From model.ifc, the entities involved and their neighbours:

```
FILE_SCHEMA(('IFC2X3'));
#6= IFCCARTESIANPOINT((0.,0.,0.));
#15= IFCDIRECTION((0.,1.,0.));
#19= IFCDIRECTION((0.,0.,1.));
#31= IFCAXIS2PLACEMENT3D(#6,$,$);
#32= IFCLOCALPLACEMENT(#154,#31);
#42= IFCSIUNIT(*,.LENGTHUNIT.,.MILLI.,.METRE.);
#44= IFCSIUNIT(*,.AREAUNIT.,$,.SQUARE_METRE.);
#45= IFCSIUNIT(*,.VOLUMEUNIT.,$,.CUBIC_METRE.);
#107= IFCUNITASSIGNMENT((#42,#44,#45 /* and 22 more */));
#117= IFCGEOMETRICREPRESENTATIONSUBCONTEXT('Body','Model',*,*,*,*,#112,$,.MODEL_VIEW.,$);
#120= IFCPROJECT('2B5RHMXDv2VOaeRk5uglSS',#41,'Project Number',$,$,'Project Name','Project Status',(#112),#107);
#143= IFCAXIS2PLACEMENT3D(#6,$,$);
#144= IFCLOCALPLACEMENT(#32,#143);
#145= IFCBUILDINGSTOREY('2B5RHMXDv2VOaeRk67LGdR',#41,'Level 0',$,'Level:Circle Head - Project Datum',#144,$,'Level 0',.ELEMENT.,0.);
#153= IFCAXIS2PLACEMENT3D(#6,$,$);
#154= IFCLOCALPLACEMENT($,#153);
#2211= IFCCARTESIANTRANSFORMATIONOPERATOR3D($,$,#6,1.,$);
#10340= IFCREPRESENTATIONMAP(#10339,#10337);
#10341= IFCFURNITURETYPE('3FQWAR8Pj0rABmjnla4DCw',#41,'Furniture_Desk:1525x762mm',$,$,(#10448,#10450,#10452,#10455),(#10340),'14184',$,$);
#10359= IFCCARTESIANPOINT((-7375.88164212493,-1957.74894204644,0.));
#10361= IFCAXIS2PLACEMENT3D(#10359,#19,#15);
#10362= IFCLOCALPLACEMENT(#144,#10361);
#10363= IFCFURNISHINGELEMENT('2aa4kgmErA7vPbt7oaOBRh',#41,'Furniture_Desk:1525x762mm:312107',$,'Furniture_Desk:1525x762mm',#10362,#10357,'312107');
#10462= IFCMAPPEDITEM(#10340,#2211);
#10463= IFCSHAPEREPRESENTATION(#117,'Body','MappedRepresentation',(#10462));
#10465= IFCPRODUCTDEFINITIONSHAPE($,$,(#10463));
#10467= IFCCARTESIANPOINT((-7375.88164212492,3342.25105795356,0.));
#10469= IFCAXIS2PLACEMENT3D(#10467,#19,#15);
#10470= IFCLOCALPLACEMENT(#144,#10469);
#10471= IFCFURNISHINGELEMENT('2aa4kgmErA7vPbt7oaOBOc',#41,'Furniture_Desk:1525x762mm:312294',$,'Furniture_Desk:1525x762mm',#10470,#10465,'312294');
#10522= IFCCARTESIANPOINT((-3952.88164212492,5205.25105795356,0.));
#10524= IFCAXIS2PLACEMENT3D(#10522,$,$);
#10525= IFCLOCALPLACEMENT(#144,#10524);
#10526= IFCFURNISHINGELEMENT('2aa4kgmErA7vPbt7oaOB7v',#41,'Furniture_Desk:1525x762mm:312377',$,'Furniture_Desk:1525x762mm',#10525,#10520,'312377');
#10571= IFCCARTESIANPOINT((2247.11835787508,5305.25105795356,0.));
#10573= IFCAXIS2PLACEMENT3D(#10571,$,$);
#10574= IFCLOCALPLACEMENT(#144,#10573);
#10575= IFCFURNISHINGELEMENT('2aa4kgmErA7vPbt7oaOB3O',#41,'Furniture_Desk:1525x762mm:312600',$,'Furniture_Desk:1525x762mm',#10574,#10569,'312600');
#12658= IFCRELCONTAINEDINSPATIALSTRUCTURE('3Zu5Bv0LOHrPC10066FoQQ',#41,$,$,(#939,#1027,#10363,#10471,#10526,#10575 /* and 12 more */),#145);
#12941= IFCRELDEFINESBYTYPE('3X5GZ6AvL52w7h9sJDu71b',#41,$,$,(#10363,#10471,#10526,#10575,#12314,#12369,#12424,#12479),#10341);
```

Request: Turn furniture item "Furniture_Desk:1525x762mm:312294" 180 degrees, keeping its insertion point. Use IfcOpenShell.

```python
import ifcopenshell
import ifcopenshell.api.geometry
import ifcopenshell.util.placement

model = ifcopenshell.open("model.ifc")

item = model.by_guid("2aa4kgmErA7vPbt7oaOBOc")
matrix = ifcopenshell.util.placement.get_local_placement(item.ObjectPlacement)
matrix = matrix @ ifcopenshell.util.placement.rotation(180, "Z")
ifcopenshell.api.geometry.edit_object_placement(model, product=item, matrix=matrix, is_si=False)

print(ifcopenshell.util.placement.get_local_placement(item.ObjectPlacement).round(3) + 0.0)

model.write("model-out.ifc")
```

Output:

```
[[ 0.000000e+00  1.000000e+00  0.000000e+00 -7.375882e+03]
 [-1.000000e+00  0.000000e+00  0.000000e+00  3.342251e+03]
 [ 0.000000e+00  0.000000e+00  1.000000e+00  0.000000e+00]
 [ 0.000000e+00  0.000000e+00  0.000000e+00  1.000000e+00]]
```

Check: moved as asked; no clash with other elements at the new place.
